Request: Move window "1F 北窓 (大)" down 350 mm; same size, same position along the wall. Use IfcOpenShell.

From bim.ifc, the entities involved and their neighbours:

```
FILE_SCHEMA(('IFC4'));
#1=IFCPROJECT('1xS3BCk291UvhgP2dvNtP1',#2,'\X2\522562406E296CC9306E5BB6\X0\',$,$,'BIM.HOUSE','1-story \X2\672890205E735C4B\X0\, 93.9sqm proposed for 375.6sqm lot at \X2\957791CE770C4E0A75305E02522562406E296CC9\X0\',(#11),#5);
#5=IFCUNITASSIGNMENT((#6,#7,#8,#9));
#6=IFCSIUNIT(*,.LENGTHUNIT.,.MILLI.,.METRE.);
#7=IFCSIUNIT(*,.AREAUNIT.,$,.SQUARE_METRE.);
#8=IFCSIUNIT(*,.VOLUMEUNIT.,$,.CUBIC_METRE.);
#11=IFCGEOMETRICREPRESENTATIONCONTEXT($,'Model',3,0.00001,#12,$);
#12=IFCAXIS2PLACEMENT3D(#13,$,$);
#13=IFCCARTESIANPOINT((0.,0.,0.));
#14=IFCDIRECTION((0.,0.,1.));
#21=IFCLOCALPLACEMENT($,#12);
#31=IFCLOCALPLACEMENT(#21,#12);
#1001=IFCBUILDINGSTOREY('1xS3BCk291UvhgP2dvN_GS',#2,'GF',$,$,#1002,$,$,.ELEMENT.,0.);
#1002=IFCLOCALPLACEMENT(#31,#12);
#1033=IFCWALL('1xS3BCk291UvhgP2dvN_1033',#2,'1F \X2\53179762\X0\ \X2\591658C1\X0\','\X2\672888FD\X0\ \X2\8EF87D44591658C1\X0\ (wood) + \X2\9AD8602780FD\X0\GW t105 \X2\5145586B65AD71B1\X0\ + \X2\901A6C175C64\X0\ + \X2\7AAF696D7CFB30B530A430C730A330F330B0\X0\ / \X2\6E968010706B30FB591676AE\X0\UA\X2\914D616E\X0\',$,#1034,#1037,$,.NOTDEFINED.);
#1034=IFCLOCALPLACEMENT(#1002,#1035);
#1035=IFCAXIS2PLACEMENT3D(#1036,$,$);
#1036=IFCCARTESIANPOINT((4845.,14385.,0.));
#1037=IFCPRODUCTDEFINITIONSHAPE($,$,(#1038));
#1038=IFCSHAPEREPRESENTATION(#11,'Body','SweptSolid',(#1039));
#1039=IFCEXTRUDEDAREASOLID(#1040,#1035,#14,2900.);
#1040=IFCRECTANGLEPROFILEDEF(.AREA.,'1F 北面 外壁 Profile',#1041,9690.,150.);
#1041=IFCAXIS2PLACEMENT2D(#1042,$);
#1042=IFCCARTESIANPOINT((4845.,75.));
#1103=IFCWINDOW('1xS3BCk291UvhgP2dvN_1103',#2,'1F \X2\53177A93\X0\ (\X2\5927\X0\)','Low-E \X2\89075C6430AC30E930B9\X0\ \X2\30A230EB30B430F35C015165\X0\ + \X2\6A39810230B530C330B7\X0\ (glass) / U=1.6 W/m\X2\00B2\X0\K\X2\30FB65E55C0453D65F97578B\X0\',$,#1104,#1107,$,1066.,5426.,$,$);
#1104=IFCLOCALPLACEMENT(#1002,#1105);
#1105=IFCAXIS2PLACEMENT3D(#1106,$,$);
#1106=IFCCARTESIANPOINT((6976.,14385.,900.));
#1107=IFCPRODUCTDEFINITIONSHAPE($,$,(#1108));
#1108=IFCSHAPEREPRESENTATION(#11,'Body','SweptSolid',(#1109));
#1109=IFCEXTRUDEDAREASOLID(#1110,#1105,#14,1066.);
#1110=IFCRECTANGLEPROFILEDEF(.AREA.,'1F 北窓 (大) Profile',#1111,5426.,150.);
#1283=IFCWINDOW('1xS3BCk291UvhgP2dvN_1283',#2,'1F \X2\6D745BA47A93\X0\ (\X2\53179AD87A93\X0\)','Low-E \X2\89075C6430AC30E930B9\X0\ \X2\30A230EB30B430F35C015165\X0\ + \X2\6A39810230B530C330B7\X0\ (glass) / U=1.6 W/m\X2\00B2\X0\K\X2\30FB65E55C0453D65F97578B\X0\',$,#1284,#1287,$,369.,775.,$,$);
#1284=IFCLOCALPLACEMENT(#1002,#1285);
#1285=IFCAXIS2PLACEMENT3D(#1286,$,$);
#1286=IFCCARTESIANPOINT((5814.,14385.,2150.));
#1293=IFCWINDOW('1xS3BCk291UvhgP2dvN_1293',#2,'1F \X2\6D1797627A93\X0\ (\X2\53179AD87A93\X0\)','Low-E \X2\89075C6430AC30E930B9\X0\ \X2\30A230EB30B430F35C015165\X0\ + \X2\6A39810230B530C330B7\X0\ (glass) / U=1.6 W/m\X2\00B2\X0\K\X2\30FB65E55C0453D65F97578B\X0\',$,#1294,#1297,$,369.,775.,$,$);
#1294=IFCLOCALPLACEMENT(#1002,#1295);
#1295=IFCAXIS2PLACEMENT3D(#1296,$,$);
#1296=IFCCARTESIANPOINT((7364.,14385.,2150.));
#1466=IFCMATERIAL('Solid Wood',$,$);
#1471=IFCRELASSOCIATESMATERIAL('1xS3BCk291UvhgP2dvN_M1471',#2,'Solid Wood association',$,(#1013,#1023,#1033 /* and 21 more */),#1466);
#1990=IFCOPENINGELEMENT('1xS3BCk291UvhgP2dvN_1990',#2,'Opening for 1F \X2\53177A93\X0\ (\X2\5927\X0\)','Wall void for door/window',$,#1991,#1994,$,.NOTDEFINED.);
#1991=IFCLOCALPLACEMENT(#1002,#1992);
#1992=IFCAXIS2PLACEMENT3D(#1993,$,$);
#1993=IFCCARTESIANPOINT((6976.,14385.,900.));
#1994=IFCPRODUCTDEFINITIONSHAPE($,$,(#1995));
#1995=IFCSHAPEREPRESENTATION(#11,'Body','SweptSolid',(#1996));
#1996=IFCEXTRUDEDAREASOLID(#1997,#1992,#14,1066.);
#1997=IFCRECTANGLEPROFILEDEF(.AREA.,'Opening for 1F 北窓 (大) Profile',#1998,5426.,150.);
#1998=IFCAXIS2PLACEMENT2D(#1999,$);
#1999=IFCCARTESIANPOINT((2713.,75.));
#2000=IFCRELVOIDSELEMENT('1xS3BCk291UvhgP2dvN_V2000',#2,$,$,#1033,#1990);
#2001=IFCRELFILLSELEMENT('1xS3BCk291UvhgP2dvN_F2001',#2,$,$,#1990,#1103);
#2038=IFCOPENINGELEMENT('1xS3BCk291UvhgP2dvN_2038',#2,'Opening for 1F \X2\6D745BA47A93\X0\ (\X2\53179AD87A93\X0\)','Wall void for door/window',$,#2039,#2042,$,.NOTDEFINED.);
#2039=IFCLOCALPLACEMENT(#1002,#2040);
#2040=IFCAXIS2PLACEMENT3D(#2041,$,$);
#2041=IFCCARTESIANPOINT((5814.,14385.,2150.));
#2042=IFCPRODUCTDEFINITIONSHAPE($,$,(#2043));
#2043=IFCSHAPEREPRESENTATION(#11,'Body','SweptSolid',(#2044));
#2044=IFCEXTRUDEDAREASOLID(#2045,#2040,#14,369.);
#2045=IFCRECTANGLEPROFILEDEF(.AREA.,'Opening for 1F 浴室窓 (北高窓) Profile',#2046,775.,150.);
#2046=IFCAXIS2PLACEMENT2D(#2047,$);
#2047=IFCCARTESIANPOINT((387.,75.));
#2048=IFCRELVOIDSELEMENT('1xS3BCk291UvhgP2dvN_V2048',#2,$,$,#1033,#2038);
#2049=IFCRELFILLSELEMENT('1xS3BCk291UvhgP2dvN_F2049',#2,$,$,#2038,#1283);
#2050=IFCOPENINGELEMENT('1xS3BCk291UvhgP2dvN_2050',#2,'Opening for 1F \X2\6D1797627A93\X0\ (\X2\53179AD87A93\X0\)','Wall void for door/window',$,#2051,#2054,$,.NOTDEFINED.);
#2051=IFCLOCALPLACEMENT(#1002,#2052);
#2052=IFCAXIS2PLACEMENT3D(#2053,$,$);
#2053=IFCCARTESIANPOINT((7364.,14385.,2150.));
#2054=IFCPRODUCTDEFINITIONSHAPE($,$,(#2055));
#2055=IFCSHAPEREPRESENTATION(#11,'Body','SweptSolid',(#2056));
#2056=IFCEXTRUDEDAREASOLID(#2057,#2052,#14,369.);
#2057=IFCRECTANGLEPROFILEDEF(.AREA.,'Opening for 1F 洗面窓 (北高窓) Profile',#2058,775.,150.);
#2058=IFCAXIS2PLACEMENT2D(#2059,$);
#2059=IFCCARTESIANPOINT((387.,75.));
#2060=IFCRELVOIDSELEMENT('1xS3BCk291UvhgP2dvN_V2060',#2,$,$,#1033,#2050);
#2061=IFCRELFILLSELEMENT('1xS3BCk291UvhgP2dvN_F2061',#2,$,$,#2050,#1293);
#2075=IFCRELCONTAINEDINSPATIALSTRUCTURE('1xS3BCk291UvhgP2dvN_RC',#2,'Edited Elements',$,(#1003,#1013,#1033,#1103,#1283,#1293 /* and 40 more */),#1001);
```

```python
import numpy as np
import ifcopenshell
import ifcopenshell.api.geometry
import ifcopenshell.util.placement
import ifcopenshell.util.unit

model = ifcopenshell.open("bim.ifc")
unit_scale = ifcopenshell.util.unit.calculate_unit_scale(model)

window = model.by_guid("1xS3BCk291UvhgP2dvN_1103")
opening = window.FillsVoids[0].RelatingOpeningElement
dz = -0.35 / unit_scale

shift = np.array([0.0, 0.0, dz])
# The window is not placed relative to its opening, so move both.
for product in (opening, window):
    matrix = ifcopenshell.util.placement.get_local_placement(product.ObjectPlacement)
    matrix[:3, 3] += shift
    ifcopenshell.api.geometry.edit_object_placement(model, product=product, matrix=matrix, is_si=False)

print(f"moved by {dz * unit_scale:+.3f} m")

model.write("bim_updated.ifc")
```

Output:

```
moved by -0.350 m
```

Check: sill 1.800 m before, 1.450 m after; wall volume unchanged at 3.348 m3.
